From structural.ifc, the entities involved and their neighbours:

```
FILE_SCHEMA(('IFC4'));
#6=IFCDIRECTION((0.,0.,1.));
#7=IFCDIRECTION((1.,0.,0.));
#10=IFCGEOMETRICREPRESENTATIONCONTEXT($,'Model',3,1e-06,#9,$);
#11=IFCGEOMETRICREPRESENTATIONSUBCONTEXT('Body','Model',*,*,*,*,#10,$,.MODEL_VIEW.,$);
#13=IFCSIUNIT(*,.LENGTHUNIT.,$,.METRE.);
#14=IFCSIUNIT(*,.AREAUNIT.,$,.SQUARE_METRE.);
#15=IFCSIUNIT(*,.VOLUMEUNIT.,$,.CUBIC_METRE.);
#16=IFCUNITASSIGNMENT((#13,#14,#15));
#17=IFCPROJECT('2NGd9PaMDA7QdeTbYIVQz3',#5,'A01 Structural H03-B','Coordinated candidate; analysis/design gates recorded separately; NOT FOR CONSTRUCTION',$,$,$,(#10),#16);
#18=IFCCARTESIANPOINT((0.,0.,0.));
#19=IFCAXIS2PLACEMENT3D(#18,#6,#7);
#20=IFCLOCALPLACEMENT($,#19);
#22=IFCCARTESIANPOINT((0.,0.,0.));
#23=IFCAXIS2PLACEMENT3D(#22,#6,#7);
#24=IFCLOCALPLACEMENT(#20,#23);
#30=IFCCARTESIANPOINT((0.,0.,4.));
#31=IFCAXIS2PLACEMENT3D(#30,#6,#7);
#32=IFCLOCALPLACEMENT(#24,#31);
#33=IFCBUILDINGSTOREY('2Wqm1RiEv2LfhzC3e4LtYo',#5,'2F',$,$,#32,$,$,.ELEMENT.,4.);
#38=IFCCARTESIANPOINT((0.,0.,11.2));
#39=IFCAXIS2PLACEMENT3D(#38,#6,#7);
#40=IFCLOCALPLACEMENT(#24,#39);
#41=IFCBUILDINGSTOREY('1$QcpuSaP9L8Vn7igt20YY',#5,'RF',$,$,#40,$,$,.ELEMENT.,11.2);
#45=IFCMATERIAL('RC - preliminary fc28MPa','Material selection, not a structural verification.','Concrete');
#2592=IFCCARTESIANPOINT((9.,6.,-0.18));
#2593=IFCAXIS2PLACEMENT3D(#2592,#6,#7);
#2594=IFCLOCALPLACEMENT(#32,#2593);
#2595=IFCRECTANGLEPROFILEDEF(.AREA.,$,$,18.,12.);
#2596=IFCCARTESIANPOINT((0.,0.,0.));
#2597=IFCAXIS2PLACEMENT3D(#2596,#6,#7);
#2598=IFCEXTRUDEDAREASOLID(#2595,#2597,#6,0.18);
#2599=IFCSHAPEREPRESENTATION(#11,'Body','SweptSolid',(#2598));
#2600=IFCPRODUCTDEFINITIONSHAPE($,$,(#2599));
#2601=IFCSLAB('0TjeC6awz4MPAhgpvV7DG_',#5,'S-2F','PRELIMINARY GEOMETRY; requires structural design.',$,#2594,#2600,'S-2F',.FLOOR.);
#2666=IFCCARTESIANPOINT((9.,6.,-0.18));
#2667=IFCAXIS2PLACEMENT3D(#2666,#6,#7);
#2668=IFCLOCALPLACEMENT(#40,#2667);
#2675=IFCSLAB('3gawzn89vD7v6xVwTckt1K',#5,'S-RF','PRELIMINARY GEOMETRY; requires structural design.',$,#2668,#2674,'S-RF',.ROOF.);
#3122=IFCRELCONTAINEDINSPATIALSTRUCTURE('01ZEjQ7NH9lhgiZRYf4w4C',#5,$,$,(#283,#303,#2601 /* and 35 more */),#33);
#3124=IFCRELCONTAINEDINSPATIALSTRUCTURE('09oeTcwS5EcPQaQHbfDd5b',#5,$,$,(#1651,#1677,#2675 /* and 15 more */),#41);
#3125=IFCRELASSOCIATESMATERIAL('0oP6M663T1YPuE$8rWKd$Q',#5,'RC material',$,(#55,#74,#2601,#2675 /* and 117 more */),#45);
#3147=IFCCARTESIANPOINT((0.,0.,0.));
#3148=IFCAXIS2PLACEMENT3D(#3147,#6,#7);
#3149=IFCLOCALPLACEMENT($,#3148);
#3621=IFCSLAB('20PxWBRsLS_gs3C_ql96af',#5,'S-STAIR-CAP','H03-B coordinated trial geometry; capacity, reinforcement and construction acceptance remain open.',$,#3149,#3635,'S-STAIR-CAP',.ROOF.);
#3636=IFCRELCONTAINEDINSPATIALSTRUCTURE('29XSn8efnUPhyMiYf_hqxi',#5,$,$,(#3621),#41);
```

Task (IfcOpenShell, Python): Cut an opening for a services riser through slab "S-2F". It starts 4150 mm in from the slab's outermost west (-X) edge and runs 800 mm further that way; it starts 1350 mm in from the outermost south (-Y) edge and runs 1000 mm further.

```python
import numpy as np
import ifcopenshell
import ifcopenshell.api.feature
import ifcopenshell.api.geometry
import ifcopenshell.api.root
import ifcopenshell.geom
import ifcopenshell.util.placement
import ifcopenshell.util.representation
import ifcopenshell.util.shape
import ifcopenshell.util.unit

model = ifcopenshell.open("structural.ifc")
unit_scale = ifcopenshell.util.unit.calculate_unit_scale(model)
settings = ifcopenshell.geom.settings()


def volume(element):
    """Net volume in cubic metres, openings subtracted."""
    shape = ifcopenshell.geom.create_shape(settings, element)
    return ifcopenshell.util.shape.get_volume(shape.geometry)


slab = model.by_guid("0TjeC6awz4MPAhgpvV7DG_")
before = volume(slab)

# Extent in the slab's own axes, in metres. The edges named are its -X and -Y sides.
slab_shape = ifcopenshell.geom.create_shape(settings, slab)
vertices = ifcopenshell.util.shape.get_vertices(slab_shape.geometry)
x_min, y_min, bottom = vertices.min(axis=0)
top = vertices[:, 2].max()

opening = ifcopenshell.api.root.create_entity(model, ifc_class="IfcOpeningElement", name="Services riser opening", predefined_type="OPENING")
context = ifcopenshell.util.representation.get_context(model, "Model", "Body", "MODEL_VIEW")
width, depth = 0.8, 1
outline = [(0.0, 0.0), (width, 0.0), (width, depth), (0.0, depth), (0.0, 0.0)]
# Overshoot both faces by 50 mm so the cut is clean.
shape = ifcopenshell.api.geometry.add_slab_representation(
    model, context=context, depth=top - bottom + 0.1, polyline=outline
)
ifcopenshell.api.geometry.assign_representation(model, product=opening, representation=shape)

matrix = ifcopenshell.util.placement.get_local_placement(slab.ObjectPlacement)
matrix[:, 3] = matrix @ np.append(np.array([x_min + 4.15, y_min + 1.35, bottom - 0.05]) / unit_scale, 1.0)
ifcopenshell.api.geometry.edit_object_placement(model, product=opening, matrix=matrix, is_si=False)
ifcopenshell.api.feature.add_feature(model, feature=opening, element=slab)

after = volume(slab)

print(f"slab volume {before:.3f} -> {after:.3f} m3")

model.write("structural_rev.ifc")
```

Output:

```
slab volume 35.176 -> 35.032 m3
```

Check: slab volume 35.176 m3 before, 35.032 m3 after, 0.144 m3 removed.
